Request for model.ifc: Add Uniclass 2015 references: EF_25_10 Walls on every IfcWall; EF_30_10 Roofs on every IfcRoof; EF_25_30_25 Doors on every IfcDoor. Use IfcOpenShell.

First a look at what the model holds.

```python
import ifcopenshell

model = ifcopenshell.open("model.ifc")
print(model.schema)
print("classifications:", [c.Name for c in model.by_type("IfcClassification")])
for ifc_class in ("IfcDoor", "IfcRoof", "IfcStair", "IfcWall", "IfcWindow"):
    print(ifc_class, len(model.by_type(ifc_class)))
```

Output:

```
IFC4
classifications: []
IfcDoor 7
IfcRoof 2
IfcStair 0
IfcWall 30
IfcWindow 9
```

```python
import ifcopenshell
import ifcopenshell.api.classification

model = ifcopenshell.open("model.ifc")

system = ifcopenshell.api.classification.add_classification(model, classification="Uniclass 2015")

codes = {
    "IfcWall": ("EF_25_10", "Walls"),
    "IfcRoof": ("EF_30_10", "Roofs"),
    "IfcDoor": ("EF_25_30_25", "Doors"),
}
for ifc_class, (code, name) in codes.items():
    products = model.by_type(ifc_class)
    ifcopenshell.api.classification.add_reference(
        model, products=products, classification=system, identification=code, name=name
    )
    print(code, len(products))

model.write("model_updated.ifc")
```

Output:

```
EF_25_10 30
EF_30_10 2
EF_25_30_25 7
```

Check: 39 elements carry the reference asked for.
